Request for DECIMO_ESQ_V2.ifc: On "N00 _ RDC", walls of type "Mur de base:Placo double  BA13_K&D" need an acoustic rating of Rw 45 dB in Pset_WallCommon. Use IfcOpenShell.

First a look at what the model holds.

```python
import ifcopenshell
import ifcopenshell.util.element

model = ifcopenshell.open("DECIMO_ESQ_V2.ifc")
print(model.schema)
storey = next(s for s in model.by_type("IfcBuildingStorey") if s.Name == "N00 _ RDC")
walls = [e for e in ifcopenshell.util.element.get_decomposition(storey) if e.is_a("IfcWall")]
seen = {}
for e in walls:
    element_type = ifcopenshell.util.element.get_type(e)
    key = (element_type.Name if element_type != e and element_type else None, ifcopenshell.util.element.get_pset(e, "Pset_WallCommon", "AcousticRating"))
    seen[key] = seen.get(key, 0) + 1
for (name, value), count in sorted(seen.items(), key=str):
    print(count, "x", name, "|", value)
```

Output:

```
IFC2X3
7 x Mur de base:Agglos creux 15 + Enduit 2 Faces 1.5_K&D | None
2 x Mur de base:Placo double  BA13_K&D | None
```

```python
import ifcopenshell
import ifcopenshell.api.pset
import ifcopenshell.util.element

model = ifcopenshell.open("DECIMO_ESQ_V2.ifc")

storey = next(s for s in model.by_type("IfcBuildingStorey") if s.Name == "N00 _ RDC")
walls = [e for e in ifcopenshell.util.element.get_decomposition(storey) if e.is_a("IfcWall")]

count = 0
for e in walls:
    element_type = ifcopenshell.util.element.get_type(e)
    if element_type in (None, e) or element_type.Name != "Mur de base:Placo double  BA13_K&D":
        continue
    # add_pset returns the element's existing set when there is one.
    pset = ifcopenshell.api.pset.add_pset(model, product=e, name="Pset_WallCommon")
    ifcopenshell.api.pset.edit_pset(model, pset=pset, properties={"AcousticRating": "Rw 45 dB"})
    count += 1

print(count, "walls updated")

model.write("DECIMO_ESQ_V2_v2.ifc")
```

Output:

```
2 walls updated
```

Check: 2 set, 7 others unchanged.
